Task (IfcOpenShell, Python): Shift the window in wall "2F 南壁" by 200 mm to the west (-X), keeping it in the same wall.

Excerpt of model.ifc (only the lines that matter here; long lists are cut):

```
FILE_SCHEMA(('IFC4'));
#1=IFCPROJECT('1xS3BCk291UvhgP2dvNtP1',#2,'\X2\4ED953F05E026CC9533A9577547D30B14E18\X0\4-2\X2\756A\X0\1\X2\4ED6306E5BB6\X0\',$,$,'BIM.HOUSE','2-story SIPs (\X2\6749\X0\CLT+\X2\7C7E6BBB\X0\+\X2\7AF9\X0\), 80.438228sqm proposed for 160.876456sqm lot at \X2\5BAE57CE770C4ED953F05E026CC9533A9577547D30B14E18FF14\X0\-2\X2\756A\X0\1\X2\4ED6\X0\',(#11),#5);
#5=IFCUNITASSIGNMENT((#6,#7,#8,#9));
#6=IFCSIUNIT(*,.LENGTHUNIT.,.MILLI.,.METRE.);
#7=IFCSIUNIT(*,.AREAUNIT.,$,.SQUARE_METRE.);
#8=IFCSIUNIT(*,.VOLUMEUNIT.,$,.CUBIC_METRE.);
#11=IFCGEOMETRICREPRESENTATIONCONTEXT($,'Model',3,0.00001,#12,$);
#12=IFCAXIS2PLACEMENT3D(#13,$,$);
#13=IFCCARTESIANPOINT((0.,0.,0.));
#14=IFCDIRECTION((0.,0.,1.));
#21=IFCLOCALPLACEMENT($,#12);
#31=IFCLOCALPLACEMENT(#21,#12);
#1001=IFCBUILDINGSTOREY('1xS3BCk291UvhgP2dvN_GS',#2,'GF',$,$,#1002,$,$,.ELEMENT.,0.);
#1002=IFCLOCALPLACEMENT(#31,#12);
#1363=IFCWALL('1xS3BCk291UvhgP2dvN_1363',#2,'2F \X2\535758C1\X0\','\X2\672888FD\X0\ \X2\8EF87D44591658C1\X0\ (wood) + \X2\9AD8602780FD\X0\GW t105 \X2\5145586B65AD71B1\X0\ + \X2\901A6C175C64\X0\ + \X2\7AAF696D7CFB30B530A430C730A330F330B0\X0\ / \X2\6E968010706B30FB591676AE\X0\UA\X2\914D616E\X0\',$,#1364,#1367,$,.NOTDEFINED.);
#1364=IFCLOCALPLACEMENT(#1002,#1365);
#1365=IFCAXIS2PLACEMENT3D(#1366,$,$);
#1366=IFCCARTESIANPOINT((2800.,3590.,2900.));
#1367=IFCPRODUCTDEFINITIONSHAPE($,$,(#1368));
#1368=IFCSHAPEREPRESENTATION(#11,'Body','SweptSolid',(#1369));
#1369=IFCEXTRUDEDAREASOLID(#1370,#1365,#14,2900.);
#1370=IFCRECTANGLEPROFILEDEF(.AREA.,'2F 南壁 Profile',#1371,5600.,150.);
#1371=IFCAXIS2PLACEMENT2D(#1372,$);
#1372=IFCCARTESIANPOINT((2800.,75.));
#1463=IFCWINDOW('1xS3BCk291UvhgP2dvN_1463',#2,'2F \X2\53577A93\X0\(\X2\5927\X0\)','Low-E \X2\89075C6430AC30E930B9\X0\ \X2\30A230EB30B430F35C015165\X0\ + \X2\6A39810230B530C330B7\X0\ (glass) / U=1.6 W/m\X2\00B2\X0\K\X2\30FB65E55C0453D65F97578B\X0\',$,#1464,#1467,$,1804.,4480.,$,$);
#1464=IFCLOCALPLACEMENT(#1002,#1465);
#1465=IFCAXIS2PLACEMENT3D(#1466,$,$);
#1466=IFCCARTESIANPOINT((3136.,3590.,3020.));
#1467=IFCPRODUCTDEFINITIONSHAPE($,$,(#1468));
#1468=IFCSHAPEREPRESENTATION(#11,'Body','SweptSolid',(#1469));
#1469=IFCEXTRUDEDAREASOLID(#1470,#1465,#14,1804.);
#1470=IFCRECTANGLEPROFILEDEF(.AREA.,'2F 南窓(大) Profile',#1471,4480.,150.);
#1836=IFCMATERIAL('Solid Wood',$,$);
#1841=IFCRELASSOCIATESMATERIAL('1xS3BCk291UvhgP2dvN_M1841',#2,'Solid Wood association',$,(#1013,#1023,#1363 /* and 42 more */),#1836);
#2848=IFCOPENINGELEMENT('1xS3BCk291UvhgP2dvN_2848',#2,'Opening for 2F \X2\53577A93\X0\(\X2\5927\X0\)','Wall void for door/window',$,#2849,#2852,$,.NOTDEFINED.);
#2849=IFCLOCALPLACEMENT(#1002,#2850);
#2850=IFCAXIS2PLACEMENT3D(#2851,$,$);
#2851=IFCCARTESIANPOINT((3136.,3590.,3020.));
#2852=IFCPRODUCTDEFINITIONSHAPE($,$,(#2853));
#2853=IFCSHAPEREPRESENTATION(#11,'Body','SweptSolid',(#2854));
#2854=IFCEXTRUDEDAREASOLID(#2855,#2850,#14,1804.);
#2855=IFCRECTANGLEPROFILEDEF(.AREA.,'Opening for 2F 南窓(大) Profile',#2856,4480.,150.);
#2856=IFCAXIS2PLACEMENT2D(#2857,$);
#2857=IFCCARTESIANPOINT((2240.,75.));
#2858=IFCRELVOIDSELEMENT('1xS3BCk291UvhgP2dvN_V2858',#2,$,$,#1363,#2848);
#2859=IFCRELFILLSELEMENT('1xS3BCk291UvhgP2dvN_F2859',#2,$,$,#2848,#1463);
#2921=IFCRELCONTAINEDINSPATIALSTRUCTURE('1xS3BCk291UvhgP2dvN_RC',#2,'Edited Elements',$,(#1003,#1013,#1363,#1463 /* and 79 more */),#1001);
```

```python
import ifcopenshell
import ifcopenshell.api.geometry
import ifcopenshell.util.placement
import ifcopenshell.util.unit

model = ifcopenshell.open("model.ifc")
unit_scale = ifcopenshell.util.unit.calculate_unit_scale(model)

window = model.by_guid("1xS3BCk291UvhgP2dvN_1463")
opening = window.FillsVoids[0].RelatingOpeningElement
wall = opening.VoidsElements[0].RelatingBuildingElement

wall_matrix = ifcopenshell.util.placement.get_local_placement(wall.ObjectPlacement)
shift = wall_matrix[:3, 0] * -0.2 / unit_scale
before = ifcopenshell.util.placement.get_local_placement(window.ObjectPlacement)[:3, 3].copy()

# The window is not placed relative to its opening, so move both.
for product in (opening, window):
    matrix = ifcopenshell.util.placement.get_local_placement(product.ObjectPlacement)
    matrix[:3, 3] += shift
    ifcopenshell.api.geometry.edit_object_placement(model, product=product, matrix=matrix, is_si=False)

after = ifcopenshell.util.placement.get_local_placement(window.ObjectPlacement)[:3, 3]
print("window moved by", (after - before).round(3) + 0.0)

model.write("model_edited.ifc")
```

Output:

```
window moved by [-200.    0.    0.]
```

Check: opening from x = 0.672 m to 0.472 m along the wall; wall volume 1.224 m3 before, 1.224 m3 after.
